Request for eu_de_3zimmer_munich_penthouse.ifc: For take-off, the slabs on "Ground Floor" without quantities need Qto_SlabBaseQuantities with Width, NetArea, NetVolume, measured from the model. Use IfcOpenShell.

First a look at what the model holds.

```python
import ifcopenshell
import ifcopenshell.util.element
import ifcopenshell.util.unit

model = ifcopenshell.open("eu_de_3zimmer_munich_penthouse.ifc")
print(model.schema)
for unit_type in ("LENGTHUNIT", "AREAUNIT", "VOLUMEUNIT"):
    print(unit_type, ifcopenshell.util.unit.calculate_unit_scale(model, unit_type))
storey = next(s for s in model.by_type("IfcBuildingStorey") if s.Name == "Ground Floor")
slabs = [e for e in ifcopenshell.util.element.get_decomposition(storey) if e.is_a("IfcSlab")]
for e in sorted(slabs, key=lambda e: e.id()):
    print(e.id(), e.is_a(), e.Name, list(ifcopenshell.util.element.get_psets(e, qtos_only=True)), sep=" | ")
```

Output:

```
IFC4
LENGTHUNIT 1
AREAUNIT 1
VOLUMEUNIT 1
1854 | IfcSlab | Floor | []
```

```python
import ifcopenshell
import ifcopenshell.api.pset
import ifcopenshell.geom
import ifcopenshell.util.element
import ifcopenshell.util.shape
import ifcopenshell.util.unit

model = ifcopenshell.open("eu_de_3zimmer_munich_penthouse.ifc")
unit_scale = ifcopenshell.util.unit.calculate_unit_scale(model)
area_scale = ifcopenshell.util.unit.calculate_unit_scale(model, "AREAUNIT")
volume_scale = ifcopenshell.util.unit.calculate_unit_scale(model, "VOLUMEUNIT")
settings = ifcopenshell.geom.settings()

storey = next(s for s in model.by_type("IfcBuildingStorey") if s.Name == "Ground Floor")
slabs = [e for e in ifcopenshell.util.element.get_decomposition(storey) if e.is_a("IfcSlab")]

for e in sorted(slabs, key=lambda e: e.id()):
    if ifcopenshell.util.element.get_psets(e, qtos_only=True, should_inherit=False):
        continue
    # Geometry comes back in metres, in the element's own axes.
    shape = ifcopenshell.geom.create_shape(settings, e)
    values = {
        "Width": ifcopenshell.util.shape.get_z(shape.geometry) / unit_scale,
        "NetArea": ifcopenshell.util.shape.get_footprint_area(shape.geometry) / area_scale,
        "NetVolume": ifcopenshell.util.shape.get_volume(shape.geometry) / volume_scale,
    }
    qto = ifcopenshell.api.pset.add_qto(model, product=e, name="Qto_SlabBaseQuantities")
    ifcopenshell.api.pset.edit_qto(model, qto=qto, properties=values)
    print(e.id(), {k: round(v, 3) for k, v in values.items()})

model.write("eu_de_3zimmer_munich_penthouse_v2.ifc")
```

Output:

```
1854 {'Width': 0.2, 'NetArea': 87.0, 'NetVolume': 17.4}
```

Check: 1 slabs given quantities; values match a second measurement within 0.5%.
